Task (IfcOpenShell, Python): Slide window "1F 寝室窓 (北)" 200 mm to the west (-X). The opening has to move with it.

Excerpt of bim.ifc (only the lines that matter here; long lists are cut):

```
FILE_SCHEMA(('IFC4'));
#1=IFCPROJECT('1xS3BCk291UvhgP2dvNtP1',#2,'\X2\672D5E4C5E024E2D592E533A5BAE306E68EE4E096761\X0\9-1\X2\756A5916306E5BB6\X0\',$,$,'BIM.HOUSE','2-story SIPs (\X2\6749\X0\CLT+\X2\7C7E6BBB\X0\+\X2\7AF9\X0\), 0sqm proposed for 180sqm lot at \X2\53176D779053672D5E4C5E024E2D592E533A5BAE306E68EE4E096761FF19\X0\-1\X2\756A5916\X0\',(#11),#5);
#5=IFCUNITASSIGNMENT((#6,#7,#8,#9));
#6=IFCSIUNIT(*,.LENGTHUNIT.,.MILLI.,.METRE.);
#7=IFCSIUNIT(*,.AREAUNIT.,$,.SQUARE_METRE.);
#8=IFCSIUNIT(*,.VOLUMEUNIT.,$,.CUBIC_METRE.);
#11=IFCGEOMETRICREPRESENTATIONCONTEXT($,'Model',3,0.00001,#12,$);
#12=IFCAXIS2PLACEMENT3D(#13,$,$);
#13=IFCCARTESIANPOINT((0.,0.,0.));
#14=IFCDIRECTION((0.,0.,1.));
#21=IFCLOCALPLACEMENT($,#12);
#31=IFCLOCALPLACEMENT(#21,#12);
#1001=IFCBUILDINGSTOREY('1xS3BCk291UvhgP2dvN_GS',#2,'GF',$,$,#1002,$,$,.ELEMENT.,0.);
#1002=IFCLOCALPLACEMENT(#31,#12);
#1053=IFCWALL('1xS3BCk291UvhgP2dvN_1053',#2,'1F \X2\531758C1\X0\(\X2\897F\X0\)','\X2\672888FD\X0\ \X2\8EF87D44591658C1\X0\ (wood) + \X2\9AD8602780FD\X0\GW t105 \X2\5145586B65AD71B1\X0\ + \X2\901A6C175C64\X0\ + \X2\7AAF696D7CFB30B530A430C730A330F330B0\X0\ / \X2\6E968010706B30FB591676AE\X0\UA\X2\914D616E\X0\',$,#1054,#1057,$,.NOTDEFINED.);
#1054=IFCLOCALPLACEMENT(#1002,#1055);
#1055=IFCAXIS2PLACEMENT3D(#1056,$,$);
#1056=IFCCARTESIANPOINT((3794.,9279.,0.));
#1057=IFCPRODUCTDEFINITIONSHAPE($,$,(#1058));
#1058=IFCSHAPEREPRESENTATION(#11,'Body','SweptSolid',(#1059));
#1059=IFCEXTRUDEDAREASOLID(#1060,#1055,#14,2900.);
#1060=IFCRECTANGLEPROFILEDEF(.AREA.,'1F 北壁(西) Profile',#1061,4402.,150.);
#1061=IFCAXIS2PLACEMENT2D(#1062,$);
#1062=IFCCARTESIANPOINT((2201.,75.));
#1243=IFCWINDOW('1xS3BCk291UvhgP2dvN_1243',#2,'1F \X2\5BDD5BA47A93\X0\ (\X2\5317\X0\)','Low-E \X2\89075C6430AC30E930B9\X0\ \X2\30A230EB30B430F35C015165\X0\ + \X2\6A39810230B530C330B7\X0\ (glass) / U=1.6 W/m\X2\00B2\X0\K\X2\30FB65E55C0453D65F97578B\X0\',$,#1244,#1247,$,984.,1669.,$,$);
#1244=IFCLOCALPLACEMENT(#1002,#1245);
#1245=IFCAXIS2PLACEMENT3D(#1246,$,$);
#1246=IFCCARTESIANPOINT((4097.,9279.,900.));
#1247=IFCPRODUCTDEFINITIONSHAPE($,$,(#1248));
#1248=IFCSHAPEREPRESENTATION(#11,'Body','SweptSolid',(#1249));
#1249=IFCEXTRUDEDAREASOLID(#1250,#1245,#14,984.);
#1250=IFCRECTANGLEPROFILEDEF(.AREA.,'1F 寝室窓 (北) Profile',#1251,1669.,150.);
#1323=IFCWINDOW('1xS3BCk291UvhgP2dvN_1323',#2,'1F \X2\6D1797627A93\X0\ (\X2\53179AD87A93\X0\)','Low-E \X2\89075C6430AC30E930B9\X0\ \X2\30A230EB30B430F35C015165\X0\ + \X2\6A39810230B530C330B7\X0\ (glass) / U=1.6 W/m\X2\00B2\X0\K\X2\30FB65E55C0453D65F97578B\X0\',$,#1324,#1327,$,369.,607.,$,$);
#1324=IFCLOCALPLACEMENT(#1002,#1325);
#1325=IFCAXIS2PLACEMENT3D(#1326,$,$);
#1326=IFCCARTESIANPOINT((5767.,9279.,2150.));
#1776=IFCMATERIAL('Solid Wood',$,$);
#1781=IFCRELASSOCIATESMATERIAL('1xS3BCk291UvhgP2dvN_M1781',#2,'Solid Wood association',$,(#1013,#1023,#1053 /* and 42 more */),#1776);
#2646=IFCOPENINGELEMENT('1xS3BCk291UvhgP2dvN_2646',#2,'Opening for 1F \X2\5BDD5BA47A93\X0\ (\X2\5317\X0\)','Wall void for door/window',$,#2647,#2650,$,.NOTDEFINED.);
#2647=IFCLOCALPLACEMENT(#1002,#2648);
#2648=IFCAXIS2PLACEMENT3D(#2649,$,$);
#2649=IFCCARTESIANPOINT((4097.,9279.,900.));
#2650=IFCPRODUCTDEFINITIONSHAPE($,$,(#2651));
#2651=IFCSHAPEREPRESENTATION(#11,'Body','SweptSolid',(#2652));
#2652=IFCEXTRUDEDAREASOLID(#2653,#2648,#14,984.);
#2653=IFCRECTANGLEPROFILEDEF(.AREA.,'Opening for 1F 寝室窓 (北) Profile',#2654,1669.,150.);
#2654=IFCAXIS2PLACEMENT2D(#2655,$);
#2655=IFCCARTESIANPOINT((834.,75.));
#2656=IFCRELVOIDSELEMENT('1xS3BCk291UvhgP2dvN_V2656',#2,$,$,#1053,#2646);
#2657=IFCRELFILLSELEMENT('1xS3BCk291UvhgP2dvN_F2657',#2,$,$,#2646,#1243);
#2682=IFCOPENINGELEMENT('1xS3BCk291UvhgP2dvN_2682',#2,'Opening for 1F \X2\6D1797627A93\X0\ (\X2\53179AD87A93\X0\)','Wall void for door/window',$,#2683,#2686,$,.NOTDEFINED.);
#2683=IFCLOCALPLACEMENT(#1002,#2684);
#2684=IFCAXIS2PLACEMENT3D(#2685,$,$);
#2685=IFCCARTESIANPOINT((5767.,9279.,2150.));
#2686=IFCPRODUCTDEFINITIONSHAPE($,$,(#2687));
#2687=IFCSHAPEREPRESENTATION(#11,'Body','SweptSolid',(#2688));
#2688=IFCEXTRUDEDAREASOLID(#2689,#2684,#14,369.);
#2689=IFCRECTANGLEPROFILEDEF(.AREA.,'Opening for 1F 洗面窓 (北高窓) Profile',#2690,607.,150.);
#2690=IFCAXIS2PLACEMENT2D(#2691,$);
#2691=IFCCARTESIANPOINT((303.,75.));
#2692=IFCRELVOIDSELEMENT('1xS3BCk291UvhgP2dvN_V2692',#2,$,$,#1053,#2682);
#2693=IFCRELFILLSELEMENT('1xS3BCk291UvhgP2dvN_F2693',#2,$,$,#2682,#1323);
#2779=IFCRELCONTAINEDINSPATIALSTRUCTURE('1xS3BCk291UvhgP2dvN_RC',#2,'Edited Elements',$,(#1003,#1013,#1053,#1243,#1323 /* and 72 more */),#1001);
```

```python
import ifcopenshell
import ifcopenshell.api.geometry
import ifcopenshell.util.placement

model = ifcopenshell.open("bim.ifc")

window = model.by_guid("1xS3BCk291UvhgP2dvN_1243")
opening = window.FillsVoids[0].RelatingOpeningElement
wall = opening.VoidsElements[0].RelatingBuildingElement

wall_matrix = ifcopenshell.util.placement.get_local_placement(wall.ObjectPlacement)
shift = wall_matrix[:3, 0] * -200.0
before = ifcopenshell.util.placement.get_local_placement(window.ObjectPlacement)[:3, 3].copy()

# The window is not placed relative to its opening, so move both.
for product in (opening, window):
    matrix = ifcopenshell.util.placement.get_local_placement(product.ObjectPlacement)
    matrix[:3, 3] += shift
    ifcopenshell.api.geometry.edit_object_placement(model, product=product, matrix=matrix, is_si=False)

after = ifcopenshell.util.placement.get_local_placement(window.ObjectPlacement)[:3, 3]
print("window moved by", (after - before).round(3) + 0.0)

model.write("bim_rev.ifc")
```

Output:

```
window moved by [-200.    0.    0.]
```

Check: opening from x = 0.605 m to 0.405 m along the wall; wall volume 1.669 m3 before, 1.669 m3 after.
